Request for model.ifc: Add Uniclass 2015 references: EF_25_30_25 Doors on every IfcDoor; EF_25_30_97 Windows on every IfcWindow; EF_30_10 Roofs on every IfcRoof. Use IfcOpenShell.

First a look at what the model holds.

```python
import ifcopenshell

model = ifcopenshell.open("model.ifc")
print(model.schema)
print("classifications:", [c.Name for c in model.by_type("IfcClassification")])
for ifc_class in ("IfcDoor", "IfcRoof", "IfcStair", "IfcWall", "IfcWindow"):
    print(ifc_class, len(model.by_type(ifc_class)))
```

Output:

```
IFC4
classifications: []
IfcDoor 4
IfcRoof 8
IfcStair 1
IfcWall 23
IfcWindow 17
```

```python
import ifcopenshell
import ifcopenshell.api.classification

model = ifcopenshell.open("model.ifc")

system = ifcopenshell.api.classification.add_classification(model, classification="Uniclass 2015")

codes = {
    "IfcDoor": ("EF_25_30_25", "Doors"),
    "IfcWindow": ("EF_25_30_97", "Windows"),
    "IfcRoof": ("EF_30_10", "Roofs"),
}
for ifc_class, (code, name) in codes.items():
    products = model.by_type(ifc_class)
    ifcopenshell.api.classification.add_reference(
        model, products=products, classification=system, identification=code, name=name
    )
    print(code, len(products))

model.write("model_v2.ifc")
```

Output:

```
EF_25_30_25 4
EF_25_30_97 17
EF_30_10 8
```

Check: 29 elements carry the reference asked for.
